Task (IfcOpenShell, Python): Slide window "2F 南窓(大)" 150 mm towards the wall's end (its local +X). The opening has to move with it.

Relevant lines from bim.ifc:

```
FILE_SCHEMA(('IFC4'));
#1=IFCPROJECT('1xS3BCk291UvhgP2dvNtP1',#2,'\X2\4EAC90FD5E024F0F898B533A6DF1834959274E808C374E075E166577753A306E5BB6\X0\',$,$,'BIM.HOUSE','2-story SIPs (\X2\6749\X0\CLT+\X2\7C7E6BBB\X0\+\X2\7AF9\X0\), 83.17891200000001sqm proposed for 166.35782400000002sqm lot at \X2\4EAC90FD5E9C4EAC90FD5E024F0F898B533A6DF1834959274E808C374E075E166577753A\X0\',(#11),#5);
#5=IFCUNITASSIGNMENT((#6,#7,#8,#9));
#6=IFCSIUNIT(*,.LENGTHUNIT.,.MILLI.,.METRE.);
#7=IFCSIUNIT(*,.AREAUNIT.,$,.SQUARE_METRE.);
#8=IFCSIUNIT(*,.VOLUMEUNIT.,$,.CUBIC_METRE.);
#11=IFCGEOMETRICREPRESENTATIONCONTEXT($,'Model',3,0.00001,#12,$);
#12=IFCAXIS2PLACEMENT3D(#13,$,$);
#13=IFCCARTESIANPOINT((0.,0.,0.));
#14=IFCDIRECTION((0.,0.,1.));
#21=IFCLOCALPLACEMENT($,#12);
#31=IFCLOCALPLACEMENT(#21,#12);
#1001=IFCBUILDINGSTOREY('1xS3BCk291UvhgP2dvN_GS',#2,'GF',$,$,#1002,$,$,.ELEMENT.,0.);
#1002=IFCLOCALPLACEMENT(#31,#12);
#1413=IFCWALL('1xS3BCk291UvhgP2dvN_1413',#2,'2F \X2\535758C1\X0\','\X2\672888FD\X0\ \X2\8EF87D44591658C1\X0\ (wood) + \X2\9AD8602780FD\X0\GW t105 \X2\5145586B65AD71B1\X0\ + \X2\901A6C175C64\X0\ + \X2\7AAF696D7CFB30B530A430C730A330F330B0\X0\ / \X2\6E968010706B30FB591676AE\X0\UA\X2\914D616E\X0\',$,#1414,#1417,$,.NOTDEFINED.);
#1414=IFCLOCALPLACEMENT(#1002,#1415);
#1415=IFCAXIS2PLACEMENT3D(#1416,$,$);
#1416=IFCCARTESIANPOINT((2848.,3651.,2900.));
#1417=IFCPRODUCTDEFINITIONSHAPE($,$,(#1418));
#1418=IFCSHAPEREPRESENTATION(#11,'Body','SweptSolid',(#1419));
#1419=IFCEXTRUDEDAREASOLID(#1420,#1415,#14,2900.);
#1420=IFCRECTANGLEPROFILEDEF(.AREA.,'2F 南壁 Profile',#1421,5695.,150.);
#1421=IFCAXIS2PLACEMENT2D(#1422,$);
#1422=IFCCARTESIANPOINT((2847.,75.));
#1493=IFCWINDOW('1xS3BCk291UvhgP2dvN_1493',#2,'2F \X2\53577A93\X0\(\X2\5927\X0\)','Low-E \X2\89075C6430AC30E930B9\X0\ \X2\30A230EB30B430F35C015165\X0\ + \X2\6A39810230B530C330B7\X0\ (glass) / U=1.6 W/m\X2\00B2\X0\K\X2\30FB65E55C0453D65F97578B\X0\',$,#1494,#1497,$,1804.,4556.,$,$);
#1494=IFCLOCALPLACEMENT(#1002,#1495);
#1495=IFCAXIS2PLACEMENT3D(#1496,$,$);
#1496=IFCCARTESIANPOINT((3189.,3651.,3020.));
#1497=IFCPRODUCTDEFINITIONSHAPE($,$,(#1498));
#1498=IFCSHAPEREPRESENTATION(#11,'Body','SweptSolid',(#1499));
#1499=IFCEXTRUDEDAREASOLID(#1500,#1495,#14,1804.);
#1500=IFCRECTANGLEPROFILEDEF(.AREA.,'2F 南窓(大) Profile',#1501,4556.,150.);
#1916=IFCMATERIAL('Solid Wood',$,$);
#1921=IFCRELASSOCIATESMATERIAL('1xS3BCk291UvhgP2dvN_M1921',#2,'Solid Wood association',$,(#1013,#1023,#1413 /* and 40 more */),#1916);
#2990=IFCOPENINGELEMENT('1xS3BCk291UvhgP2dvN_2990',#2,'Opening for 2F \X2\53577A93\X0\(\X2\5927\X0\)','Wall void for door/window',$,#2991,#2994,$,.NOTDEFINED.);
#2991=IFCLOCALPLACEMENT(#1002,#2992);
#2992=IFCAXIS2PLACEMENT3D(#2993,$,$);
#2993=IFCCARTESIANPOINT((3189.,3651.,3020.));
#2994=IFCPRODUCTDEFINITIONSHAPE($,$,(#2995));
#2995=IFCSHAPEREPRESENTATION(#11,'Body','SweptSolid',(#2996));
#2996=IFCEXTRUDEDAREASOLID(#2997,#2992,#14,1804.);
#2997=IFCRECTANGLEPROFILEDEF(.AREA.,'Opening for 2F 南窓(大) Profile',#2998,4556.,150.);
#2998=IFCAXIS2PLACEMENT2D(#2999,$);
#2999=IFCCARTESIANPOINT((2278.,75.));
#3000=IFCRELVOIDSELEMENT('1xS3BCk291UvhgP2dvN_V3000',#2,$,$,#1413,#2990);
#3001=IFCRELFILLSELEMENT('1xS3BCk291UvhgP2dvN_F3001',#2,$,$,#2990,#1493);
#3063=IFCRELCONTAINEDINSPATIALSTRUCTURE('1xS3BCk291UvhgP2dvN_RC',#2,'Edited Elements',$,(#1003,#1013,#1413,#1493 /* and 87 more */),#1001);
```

```python
import ifcopenshell
import ifcopenshell.api.geometry
import ifcopenshell.util.placement
import ifcopenshell.util.unit

model = ifcopenshell.open("bim.ifc")
unit_scale = ifcopenshell.util.unit.calculate_unit_scale(model)

window = model.by_id(1493)
opening = window.FillsVoids[0].RelatingOpeningElement
wall = opening.VoidsElements[0].RelatingBuildingElement

wall_matrix = ifcopenshell.util.placement.get_local_placement(wall.ObjectPlacement)
shift = wall_matrix[:3, 0] * 0.15 / unit_scale
before = ifcopenshell.util.placement.get_local_placement(window.ObjectPlacement)[:3, 3].copy()

# The window is not placed relative to its opening, so move both.
for product in (opening, window):
    matrix = ifcopenshell.util.placement.get_local_placement(product.ObjectPlacement)
    matrix[:3, 3] += shift
    ifcopenshell.api.geometry.edit_object_placement(model, product=product, matrix=matrix, is_si=False)

after = ifcopenshell.util.placement.get_local_placement(window.ObjectPlacement)[:3, 3]
print("window moved by", (after - before).round(3) + 0.0)

model.write("bim_v2.ifc")
```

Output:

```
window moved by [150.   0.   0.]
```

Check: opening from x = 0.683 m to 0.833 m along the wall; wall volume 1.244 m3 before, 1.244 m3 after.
